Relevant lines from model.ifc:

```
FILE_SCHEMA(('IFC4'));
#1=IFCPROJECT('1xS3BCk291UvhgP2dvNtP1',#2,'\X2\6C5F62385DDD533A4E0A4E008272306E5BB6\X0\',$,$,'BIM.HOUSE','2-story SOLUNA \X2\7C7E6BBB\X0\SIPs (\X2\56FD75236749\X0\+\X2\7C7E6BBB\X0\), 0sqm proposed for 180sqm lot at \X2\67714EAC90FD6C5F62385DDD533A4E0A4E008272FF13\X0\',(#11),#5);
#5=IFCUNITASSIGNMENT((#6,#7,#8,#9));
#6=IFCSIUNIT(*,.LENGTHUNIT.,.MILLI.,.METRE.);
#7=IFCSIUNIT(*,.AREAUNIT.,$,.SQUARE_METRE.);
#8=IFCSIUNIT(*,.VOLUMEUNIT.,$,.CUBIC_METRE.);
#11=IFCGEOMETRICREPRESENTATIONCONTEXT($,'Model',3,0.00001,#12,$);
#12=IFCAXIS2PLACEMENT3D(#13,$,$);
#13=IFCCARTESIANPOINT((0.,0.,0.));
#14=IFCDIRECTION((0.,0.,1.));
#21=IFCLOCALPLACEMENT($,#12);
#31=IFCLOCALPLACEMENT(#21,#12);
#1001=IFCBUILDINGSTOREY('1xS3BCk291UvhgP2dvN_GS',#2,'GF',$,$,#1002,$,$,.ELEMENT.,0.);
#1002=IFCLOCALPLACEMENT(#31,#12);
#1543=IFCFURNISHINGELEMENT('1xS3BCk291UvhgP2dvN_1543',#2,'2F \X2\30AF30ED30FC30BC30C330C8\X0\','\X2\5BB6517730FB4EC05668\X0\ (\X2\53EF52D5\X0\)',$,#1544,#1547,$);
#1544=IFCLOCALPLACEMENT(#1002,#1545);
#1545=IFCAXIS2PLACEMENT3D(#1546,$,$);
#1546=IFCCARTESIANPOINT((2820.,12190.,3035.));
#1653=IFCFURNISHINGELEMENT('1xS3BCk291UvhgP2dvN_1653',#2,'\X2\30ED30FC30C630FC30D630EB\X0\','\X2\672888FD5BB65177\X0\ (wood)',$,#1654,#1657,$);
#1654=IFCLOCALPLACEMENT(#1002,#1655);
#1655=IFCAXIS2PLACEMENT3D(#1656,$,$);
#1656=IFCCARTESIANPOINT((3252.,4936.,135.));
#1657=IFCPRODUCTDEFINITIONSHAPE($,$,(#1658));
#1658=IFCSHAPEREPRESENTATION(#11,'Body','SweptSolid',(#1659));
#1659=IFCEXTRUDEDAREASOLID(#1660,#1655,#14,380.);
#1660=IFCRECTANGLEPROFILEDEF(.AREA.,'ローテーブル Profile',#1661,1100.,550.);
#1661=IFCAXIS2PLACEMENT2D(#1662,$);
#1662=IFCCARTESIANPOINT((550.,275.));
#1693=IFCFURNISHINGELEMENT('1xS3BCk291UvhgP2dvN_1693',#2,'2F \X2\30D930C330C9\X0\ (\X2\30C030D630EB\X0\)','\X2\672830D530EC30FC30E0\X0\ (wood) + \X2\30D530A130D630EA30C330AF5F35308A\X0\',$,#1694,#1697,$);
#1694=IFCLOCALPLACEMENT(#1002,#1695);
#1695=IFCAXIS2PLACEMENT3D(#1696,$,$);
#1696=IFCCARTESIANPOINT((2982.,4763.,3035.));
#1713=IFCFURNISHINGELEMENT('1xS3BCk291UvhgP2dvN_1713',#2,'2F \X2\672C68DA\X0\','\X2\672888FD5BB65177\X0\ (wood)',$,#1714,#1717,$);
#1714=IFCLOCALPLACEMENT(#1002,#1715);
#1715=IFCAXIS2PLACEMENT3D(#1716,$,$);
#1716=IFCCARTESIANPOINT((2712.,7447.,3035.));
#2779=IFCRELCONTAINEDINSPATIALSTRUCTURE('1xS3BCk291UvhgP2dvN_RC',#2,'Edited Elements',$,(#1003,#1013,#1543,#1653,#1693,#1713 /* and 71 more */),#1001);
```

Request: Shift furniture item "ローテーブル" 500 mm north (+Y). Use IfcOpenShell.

```python
import ifcopenshell
import ifcopenshell.api.geometry
import ifcopenshell.util.placement
import ifcopenshell.util.unit

model = ifcopenshell.open("model.ifc")
unit_scale = ifcopenshell.util.unit.calculate_unit_scale(model)

item = model.by_guid("1xS3BCk291UvhgP2dvN_1653")
matrix = ifcopenshell.util.placement.get_local_placement(item.ObjectPlacement)
matrix[1, 3] += 0.5 / unit_scale
ifcopenshell.api.geometry.edit_object_placement(model, product=item, matrix=matrix, is_si=False)

print(ifcopenshell.util.placement.get_local_placement(item.ObjectPlacement).round(3) + 0.0)

model.write("model-out.ifc")
```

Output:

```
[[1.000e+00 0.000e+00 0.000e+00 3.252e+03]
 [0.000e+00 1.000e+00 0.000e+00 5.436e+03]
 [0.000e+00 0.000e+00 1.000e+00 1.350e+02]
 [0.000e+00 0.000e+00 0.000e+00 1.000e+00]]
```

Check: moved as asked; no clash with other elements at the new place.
